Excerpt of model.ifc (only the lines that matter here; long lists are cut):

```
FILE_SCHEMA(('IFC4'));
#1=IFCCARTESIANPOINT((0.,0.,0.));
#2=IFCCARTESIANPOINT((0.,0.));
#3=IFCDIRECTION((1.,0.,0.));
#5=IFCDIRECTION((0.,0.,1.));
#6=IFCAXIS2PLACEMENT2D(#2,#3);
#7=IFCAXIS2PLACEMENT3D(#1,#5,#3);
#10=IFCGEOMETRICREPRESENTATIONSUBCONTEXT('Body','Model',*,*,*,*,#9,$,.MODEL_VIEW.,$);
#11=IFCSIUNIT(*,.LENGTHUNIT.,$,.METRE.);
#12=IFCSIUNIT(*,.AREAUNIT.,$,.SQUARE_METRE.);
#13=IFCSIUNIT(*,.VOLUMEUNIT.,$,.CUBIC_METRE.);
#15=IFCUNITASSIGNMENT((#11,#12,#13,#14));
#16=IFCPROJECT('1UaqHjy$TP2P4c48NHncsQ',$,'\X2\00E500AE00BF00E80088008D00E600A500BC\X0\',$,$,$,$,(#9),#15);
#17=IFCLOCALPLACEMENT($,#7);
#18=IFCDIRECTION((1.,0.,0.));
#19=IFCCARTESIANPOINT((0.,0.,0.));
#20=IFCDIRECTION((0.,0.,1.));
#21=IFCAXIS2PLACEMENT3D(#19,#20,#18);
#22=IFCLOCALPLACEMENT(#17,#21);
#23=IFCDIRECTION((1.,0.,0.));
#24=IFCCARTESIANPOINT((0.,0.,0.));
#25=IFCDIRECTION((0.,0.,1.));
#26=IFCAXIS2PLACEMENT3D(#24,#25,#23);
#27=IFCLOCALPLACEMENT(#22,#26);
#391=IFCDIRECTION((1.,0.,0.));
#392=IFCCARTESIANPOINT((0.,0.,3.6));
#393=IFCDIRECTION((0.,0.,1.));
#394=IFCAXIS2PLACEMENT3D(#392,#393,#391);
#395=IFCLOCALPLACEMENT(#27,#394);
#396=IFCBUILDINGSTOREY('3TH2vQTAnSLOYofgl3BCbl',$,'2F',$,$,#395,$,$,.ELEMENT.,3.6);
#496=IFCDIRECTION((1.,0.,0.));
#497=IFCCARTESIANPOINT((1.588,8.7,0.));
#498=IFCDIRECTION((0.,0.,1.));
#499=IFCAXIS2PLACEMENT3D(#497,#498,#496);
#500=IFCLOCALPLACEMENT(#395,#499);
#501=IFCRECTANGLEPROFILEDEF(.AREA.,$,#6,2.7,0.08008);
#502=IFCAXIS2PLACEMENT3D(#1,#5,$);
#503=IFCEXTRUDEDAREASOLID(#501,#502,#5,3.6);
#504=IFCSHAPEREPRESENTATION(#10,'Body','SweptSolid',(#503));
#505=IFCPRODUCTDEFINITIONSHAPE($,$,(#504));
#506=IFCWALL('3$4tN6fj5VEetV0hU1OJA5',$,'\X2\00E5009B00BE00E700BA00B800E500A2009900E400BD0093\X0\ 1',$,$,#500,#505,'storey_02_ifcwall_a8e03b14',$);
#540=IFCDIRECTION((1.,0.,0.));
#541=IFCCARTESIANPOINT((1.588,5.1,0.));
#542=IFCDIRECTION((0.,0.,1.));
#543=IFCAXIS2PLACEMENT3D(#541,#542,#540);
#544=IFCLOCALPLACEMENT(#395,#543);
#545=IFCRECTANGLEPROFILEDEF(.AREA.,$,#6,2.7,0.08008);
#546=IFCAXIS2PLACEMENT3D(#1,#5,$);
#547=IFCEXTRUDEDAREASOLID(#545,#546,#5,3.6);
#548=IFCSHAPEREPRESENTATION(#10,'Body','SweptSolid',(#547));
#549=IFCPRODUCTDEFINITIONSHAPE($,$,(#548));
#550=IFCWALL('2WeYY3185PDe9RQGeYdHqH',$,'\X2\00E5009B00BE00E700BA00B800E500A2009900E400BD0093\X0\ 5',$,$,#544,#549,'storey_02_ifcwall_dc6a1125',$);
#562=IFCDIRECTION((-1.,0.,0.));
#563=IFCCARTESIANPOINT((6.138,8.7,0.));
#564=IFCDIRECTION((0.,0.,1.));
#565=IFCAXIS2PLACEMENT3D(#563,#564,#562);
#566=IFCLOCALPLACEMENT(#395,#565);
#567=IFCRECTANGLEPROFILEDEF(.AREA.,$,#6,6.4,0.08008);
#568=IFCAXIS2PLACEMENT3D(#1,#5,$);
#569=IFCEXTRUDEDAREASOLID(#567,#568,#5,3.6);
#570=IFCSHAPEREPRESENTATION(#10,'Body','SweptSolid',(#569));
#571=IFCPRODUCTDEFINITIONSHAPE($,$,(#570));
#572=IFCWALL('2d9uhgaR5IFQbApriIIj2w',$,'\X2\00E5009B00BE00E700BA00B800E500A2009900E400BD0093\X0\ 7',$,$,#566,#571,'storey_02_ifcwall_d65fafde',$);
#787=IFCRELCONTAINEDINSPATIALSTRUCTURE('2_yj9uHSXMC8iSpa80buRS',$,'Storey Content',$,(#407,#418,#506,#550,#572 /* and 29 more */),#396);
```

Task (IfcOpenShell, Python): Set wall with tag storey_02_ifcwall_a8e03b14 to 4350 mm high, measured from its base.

```python
import ifcopenshell
import ifcopenshell.geom
import ifcopenshell.util.representation
import ifcopenshell.util.shape

model = ifcopenshell.open("model.ifc")
settings = ifcopenshell.geom.settings()


def volume(element):
    """Net volume in cubic metres, openings subtracted."""
    shape = ifcopenshell.geom.create_shape(settings, element)
    return ifcopenshell.util.shape.get_volume(shape.geometry)


wall = model.by_id(506)
before = volume(wall)

body = ifcopenshell.util.representation.get_representation(wall, "Model", "Body")
solid = body.Items[0]
old_height = solid.Depth
solid.Depth = 4.35
after = volume(wall)

print(f"height {old_height:g} -> {solid.Depth:g}, volume {before:.3f} -> {after:.3f} m3")

model.write("model_rev.ifc")
```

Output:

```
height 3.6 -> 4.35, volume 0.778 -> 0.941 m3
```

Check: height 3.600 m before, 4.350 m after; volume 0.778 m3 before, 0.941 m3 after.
